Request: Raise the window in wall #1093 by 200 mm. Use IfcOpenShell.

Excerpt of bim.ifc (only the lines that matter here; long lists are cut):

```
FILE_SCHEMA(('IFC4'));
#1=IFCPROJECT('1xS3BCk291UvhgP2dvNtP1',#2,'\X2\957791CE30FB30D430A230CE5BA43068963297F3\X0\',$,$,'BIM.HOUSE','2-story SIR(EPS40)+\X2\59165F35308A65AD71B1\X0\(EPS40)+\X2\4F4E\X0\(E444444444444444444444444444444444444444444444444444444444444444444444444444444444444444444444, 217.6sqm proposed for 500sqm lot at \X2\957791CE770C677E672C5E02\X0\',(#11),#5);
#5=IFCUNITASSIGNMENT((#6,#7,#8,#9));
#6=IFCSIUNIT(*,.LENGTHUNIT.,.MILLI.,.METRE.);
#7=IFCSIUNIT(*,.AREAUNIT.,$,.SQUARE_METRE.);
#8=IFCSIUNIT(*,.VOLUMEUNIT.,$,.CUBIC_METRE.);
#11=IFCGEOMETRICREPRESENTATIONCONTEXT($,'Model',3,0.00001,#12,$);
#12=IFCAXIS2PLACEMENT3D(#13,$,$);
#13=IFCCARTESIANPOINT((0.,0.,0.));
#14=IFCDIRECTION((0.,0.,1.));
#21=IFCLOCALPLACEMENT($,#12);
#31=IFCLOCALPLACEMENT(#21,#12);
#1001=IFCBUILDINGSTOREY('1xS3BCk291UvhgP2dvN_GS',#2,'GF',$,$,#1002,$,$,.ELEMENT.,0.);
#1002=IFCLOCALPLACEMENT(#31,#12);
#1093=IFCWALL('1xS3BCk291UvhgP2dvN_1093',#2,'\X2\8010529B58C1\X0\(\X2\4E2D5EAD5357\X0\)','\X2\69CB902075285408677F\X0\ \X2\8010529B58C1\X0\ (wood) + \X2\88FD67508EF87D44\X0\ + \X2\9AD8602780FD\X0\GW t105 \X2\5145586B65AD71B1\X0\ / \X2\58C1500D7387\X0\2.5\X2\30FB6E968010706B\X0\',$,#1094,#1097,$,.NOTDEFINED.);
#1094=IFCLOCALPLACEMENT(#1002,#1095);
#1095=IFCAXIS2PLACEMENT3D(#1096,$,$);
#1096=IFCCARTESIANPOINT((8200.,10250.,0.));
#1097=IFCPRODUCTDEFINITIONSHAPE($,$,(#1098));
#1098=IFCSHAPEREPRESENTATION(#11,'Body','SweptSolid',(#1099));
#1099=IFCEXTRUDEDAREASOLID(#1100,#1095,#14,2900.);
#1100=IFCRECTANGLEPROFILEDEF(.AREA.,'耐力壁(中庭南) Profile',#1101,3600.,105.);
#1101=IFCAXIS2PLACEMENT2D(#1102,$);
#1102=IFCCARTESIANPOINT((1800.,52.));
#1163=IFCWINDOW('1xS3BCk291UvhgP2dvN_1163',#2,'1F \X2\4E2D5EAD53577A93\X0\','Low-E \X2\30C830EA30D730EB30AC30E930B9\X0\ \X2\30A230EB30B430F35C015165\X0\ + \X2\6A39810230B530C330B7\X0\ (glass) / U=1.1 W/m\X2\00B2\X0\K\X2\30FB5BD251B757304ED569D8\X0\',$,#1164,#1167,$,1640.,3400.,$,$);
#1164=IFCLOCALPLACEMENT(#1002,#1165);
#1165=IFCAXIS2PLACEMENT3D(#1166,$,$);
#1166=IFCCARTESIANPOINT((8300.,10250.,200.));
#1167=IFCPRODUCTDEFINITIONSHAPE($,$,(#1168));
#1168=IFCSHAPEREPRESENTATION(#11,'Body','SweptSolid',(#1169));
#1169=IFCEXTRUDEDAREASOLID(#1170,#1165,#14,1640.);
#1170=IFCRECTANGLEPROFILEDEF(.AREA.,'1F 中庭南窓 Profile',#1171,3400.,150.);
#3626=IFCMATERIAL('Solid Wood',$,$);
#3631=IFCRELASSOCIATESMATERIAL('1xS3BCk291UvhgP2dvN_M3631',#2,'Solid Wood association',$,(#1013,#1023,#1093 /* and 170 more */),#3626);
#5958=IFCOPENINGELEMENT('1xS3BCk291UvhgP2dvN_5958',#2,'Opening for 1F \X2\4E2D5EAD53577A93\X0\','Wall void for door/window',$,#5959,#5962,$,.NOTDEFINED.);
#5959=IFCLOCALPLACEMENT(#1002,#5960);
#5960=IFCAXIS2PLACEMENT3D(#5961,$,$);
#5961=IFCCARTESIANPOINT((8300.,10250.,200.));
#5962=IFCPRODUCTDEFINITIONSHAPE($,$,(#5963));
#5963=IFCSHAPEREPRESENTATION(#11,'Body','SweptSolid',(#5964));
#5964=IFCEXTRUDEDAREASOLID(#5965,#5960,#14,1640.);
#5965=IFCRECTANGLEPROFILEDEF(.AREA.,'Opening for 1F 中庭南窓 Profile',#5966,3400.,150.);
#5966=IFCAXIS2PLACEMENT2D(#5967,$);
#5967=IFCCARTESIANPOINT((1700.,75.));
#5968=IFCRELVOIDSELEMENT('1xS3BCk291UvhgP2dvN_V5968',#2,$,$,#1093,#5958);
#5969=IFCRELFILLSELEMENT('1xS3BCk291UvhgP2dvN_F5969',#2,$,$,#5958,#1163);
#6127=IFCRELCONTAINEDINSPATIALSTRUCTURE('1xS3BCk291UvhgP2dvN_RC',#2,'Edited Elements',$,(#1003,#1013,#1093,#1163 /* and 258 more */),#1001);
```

```python
import numpy as np
import ifcopenshell
import ifcopenshell.api.geometry
import ifcopenshell.util.placement
import ifcopenshell.util.unit

model = ifcopenshell.open("bim.ifc")
unit_scale = ifcopenshell.util.unit.calculate_unit_scale(model)

window = model.by_guid("1xS3BCk291UvhgP2dvN_1163")
opening = window.FillsVoids[0].RelatingOpeningElement
dz = 200.0

shift = np.array([0.0, 0.0, dz])
# The window is not placed relative to its opening, so move both.
for product in (opening, window):
    matrix = ifcopenshell.util.placement.get_local_placement(product.ObjectPlacement)
    matrix[:3, 3] += shift
    ifcopenshell.api.geometry.edit_object_placement(model, product=product, matrix=matrix, is_si=False)

print(f"moved by {dz * unit_scale:+.3f} m")

model.write("bim_v2.ifc")
```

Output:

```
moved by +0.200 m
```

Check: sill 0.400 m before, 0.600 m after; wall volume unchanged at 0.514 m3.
